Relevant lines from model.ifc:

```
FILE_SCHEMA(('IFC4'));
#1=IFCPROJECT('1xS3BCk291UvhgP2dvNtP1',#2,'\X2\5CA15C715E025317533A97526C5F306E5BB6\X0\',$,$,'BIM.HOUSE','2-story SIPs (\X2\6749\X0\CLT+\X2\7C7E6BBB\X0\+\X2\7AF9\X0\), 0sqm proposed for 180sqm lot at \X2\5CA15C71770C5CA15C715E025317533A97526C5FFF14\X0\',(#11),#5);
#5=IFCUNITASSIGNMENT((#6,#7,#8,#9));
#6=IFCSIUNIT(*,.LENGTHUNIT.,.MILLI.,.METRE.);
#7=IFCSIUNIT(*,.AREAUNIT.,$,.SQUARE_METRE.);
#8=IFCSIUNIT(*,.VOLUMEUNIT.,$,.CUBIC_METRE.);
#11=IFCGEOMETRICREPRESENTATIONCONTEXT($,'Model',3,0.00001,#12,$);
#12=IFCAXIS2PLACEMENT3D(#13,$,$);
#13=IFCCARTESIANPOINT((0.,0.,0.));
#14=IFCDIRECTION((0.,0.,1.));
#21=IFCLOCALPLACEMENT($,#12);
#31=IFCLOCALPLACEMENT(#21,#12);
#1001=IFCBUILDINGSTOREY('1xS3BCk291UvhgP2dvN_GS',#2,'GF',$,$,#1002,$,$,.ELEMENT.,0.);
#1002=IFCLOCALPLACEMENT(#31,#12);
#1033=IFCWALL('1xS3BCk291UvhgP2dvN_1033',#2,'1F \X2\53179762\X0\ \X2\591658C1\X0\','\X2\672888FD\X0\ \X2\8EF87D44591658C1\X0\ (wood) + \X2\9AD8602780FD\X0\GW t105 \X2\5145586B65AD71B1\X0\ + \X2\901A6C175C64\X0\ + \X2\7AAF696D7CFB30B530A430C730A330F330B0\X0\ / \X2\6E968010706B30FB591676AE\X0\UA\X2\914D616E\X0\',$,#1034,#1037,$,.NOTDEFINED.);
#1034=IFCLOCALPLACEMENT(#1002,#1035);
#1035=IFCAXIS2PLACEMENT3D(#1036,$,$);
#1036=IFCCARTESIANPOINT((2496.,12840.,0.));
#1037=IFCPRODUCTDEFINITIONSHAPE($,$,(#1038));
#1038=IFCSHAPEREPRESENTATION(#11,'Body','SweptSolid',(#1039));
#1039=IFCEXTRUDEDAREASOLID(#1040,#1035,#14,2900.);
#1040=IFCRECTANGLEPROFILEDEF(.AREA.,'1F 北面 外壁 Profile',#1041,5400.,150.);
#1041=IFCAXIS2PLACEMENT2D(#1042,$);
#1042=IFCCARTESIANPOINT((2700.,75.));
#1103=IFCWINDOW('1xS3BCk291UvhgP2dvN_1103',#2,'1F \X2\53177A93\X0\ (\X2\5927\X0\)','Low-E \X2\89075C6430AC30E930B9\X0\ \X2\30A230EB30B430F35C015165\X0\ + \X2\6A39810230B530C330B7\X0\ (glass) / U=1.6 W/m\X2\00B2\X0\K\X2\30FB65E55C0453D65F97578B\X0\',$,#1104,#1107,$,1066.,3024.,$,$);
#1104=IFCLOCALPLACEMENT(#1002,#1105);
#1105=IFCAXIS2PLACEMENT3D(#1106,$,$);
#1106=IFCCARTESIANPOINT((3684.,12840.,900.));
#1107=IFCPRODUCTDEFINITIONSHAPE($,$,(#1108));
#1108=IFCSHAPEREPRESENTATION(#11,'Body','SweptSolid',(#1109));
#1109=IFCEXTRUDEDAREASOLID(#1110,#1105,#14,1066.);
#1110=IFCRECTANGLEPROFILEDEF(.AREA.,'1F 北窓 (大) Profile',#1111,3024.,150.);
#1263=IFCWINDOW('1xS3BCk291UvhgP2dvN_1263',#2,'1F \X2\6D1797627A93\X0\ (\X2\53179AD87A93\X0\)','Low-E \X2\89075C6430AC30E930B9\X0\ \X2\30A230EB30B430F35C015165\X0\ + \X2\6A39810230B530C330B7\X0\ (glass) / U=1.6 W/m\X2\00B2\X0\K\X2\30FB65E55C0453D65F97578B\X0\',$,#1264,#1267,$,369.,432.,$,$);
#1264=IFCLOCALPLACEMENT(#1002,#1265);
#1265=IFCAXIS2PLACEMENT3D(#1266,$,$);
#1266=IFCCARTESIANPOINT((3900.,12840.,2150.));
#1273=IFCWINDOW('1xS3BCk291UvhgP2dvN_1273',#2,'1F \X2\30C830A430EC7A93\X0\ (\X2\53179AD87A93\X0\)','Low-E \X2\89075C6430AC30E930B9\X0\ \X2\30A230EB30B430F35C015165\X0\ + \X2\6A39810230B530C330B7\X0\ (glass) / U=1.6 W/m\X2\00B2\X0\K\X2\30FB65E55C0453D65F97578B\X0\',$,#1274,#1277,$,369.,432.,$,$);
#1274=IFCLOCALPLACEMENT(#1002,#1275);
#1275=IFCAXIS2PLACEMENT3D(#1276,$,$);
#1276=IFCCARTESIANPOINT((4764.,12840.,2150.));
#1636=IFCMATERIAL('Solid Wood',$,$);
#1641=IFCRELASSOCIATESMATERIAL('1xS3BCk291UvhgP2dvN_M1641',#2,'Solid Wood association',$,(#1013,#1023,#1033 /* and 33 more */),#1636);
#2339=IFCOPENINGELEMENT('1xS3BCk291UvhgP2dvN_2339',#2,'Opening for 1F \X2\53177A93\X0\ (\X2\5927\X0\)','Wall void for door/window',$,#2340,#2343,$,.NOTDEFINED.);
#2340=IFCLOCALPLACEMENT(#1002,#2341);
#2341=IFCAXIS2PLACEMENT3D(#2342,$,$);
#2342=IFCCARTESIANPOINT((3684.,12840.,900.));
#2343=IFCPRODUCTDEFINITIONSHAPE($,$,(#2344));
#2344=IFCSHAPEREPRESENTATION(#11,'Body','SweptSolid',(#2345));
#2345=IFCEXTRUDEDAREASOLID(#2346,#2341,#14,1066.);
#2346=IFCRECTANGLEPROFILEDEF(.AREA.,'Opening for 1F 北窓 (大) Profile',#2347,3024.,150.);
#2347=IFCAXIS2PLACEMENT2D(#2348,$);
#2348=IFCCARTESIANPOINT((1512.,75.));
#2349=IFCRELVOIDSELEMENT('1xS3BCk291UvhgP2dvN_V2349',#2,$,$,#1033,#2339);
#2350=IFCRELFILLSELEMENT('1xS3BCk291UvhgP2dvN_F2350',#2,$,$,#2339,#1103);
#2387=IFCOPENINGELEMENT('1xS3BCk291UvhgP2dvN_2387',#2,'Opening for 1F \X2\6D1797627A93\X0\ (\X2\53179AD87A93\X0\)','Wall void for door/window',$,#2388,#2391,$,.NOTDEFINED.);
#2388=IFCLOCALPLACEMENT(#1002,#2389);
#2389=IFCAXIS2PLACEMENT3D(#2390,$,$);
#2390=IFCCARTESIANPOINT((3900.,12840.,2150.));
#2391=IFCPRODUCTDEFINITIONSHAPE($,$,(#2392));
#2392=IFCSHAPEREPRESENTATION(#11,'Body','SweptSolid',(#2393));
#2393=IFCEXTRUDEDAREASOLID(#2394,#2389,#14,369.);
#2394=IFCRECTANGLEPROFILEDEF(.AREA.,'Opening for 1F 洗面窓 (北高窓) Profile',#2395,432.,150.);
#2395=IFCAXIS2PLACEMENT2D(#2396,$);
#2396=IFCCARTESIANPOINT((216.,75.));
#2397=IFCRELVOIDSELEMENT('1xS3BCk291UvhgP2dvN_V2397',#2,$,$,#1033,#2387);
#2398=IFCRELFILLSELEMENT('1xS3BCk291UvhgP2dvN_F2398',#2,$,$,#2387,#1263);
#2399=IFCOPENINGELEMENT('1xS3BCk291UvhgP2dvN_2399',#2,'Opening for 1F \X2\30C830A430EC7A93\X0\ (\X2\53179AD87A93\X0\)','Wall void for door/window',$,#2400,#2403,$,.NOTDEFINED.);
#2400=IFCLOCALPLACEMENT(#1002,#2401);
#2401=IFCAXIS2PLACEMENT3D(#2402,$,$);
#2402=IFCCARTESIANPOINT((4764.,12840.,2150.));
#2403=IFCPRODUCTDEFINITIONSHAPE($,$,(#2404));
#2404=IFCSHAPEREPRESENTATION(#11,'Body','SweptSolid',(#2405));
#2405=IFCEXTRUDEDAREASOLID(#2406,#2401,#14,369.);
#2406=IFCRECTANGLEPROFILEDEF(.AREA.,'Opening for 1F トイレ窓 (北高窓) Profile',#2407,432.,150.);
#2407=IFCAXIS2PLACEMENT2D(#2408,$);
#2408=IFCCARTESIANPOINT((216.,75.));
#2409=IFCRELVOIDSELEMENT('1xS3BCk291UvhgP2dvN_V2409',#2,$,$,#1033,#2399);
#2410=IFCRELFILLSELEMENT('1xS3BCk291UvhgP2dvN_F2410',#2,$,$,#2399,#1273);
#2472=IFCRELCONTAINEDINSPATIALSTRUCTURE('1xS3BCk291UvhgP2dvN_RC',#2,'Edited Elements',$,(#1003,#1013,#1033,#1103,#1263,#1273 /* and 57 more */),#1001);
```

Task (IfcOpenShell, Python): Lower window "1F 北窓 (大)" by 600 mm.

```python
import numpy as np
import ifcopenshell
import ifcopenshell.api.geometry
import ifcopenshell.util.placement
import ifcopenshell.util.unit

model = ifcopenshell.open("model.ifc")
unit_scale = ifcopenshell.util.unit.calculate_unit_scale(model)

window = model.by_guid("1xS3BCk291UvhgP2dvN_1103")
opening = window.FillsVoids[0].RelatingOpeningElement
dz = -600.0

shift = np.array([0.0, 0.0, dz])
# The window is not placed relative to its opening, so move both.
for product in (opening, window):
    matrix = ifcopenshell.util.placement.get_local_placement(product.ObjectPlacement)
    matrix[:3, 3] += shift
    ifcopenshell.api.geometry.edit_object_placement(model, product=product, matrix=matrix, is_si=False)

print(f"moved by {dz * unit_scale:+.3f} m")

model.write("model_rev.ifc")
```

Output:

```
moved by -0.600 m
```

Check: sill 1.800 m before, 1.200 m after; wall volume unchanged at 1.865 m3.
